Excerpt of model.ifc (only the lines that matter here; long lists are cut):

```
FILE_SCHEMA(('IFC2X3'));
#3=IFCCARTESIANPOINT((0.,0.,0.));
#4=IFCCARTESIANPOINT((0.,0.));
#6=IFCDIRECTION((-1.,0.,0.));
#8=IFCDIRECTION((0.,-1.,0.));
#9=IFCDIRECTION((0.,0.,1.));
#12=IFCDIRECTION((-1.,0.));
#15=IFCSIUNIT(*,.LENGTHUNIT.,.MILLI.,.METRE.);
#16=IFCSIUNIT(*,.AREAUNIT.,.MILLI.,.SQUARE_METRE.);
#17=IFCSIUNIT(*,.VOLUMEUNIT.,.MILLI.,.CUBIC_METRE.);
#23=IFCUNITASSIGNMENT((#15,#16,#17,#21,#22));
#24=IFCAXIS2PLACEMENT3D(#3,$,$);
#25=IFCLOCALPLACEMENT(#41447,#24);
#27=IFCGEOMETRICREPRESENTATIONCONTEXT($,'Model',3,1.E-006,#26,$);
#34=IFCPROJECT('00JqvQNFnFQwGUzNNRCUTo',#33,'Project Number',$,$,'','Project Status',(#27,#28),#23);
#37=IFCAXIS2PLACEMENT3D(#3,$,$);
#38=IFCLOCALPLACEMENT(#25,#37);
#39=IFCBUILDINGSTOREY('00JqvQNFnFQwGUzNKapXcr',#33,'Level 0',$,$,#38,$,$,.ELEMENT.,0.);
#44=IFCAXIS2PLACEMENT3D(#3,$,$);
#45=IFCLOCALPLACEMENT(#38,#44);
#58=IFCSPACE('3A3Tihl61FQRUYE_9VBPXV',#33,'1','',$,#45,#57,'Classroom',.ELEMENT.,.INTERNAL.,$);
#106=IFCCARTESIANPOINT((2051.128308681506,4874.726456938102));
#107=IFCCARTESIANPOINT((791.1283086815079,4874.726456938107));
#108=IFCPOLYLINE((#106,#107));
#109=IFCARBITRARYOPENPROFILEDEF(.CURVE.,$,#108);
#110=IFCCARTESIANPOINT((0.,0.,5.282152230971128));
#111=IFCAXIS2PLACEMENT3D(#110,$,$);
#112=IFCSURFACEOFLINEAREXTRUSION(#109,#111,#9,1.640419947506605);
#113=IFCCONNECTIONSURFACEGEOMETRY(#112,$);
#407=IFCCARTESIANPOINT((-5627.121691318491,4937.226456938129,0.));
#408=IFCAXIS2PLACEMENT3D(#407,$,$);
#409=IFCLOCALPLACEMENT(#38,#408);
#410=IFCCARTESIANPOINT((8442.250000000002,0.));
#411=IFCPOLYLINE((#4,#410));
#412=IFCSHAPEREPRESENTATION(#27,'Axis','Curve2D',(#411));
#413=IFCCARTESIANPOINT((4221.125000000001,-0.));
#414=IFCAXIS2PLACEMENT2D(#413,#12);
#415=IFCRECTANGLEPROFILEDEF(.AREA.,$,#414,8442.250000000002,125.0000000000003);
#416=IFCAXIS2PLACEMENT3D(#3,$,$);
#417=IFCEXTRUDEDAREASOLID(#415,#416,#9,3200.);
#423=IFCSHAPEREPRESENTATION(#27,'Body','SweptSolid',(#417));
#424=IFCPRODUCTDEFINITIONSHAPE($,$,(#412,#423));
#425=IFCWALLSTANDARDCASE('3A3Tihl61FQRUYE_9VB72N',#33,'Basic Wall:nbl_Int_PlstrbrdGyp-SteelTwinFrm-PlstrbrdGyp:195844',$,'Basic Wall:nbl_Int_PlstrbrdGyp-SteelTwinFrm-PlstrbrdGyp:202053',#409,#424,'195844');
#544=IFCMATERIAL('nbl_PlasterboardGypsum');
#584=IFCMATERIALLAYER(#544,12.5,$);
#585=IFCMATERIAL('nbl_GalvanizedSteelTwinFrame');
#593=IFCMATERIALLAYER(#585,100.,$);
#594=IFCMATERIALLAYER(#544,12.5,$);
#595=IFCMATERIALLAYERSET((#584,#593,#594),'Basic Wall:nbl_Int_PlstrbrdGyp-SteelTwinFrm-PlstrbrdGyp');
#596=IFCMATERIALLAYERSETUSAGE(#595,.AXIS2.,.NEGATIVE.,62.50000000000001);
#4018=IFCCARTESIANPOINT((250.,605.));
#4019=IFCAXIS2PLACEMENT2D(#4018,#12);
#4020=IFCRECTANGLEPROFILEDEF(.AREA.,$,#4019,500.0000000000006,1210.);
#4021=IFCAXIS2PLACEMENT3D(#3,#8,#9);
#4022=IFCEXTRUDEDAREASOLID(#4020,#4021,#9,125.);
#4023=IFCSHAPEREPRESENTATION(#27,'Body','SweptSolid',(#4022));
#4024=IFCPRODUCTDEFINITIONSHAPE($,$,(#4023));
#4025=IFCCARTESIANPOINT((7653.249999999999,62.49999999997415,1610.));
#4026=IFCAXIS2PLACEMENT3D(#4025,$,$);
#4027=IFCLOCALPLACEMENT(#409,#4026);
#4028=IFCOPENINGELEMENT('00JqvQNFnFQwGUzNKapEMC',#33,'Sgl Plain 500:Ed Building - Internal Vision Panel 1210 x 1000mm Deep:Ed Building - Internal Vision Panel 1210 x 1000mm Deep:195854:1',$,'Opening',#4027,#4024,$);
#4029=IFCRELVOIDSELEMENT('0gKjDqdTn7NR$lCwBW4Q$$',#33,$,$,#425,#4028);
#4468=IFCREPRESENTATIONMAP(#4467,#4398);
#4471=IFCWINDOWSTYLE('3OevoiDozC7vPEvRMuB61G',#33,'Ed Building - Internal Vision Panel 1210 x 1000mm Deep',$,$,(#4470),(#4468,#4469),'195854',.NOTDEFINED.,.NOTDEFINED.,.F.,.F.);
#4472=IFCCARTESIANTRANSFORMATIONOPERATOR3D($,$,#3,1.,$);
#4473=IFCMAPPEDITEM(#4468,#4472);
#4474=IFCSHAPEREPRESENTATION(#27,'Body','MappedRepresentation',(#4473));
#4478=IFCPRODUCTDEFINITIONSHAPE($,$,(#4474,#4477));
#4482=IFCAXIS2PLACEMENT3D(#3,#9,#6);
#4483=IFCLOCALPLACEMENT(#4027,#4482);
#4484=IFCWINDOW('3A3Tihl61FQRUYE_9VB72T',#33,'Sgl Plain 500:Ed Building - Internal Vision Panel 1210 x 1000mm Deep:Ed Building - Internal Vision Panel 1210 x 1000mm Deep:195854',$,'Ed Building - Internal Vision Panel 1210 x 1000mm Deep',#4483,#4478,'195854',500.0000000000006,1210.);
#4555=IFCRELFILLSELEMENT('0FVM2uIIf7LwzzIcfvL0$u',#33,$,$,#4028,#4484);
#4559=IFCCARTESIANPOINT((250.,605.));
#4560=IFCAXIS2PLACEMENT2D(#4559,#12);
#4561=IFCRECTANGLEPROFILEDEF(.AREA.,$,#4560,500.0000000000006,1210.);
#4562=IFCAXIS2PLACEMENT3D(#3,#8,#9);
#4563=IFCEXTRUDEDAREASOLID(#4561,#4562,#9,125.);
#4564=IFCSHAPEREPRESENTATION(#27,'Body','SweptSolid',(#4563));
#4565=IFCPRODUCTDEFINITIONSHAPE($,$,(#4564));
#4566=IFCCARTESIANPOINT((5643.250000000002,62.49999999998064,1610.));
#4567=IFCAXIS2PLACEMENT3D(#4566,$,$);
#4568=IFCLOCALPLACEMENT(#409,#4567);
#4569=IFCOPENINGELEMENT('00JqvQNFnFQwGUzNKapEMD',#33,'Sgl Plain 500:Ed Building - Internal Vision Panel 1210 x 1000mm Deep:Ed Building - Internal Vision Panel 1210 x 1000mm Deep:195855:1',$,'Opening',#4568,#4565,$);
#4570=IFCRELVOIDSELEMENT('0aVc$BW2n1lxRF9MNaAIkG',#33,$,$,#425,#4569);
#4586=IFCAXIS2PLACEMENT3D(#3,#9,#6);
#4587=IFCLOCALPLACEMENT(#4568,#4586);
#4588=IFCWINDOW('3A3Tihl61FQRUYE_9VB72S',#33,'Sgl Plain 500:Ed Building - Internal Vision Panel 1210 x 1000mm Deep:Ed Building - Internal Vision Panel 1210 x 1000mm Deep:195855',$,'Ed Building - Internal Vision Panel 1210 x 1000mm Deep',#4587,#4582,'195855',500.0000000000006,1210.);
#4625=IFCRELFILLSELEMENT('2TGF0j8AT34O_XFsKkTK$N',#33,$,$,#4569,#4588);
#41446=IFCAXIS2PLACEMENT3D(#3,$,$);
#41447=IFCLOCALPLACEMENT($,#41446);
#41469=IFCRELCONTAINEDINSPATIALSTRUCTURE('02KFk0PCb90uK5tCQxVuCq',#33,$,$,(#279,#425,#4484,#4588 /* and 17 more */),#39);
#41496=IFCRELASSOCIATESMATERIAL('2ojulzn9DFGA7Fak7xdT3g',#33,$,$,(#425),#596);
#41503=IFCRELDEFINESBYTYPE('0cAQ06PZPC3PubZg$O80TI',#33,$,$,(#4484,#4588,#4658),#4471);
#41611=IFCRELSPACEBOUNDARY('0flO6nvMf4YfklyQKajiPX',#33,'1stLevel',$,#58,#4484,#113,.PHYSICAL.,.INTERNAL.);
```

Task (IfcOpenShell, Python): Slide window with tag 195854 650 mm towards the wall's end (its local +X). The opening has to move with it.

```python
import numpy as np
import ifcopenshell
import ifcopenshell.api.geometry
import ifcopenshell.util.placement
import ifcopenshell.util.unit

model = ifcopenshell.open("model.ifc")
unit_scale = ifcopenshell.util.unit.calculate_unit_scale(model)

window = model.by_guid("3A3Tihl61FQRUYE_9VB72T")
opening = window.FillsVoids[0].RelatingOpeningElement
wall = opening.VoidsElements[0].RelatingBuildingElement

wall_matrix = ifcopenshell.util.placement.get_local_placement(wall.ObjectPlacement)
shift = wall_matrix[:3, 0] * 0.65 / unit_scale
before = ifcopenshell.util.placement.get_local_placement(window.ObjectPlacement)[:3, 3].copy()

# The window is placed relative to its opening, so it follows when the opening moves.
matrix = ifcopenshell.util.placement.get_local_placement(opening.ObjectPlacement)
matrix[:3, 3] += shift
ifcopenshell.api.geometry.edit_object_placement(
    model, product=opening, matrix=matrix, is_si=False, should_transform_children=True
)

# Space boundary surfaces are stored in each space's coordinates; move them too.
for rel in window.ProvidesBoundaries:
    if not rel.ConnectionGeometry:
        continue
    surface = rel.ConnectionGeometry.SurfaceOnRelatingElement
    space_matrix = ifcopenshell.util.placement.get_local_placement(rel.RelatingSpace.ObjectPlacement)
    point = np.array(surface.Position.Location.Coordinates) + space_matrix[:3, :3].T @ shift
    surface.Position = model.createIfcAxis2Placement3D(
        model.createIfcCartesianPoint(point.tolist()), surface.Position.Axis, surface.Position.RefDirection
    )

after = ifcopenshell.util.placement.get_local_placement(window.ObjectPlacement)[:3, 3]
print("window moved by", (after - before).round(3) + 0.0)

model.write("model-out.ifc")
```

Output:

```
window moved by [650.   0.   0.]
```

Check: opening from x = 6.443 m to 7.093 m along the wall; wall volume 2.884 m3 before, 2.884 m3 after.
